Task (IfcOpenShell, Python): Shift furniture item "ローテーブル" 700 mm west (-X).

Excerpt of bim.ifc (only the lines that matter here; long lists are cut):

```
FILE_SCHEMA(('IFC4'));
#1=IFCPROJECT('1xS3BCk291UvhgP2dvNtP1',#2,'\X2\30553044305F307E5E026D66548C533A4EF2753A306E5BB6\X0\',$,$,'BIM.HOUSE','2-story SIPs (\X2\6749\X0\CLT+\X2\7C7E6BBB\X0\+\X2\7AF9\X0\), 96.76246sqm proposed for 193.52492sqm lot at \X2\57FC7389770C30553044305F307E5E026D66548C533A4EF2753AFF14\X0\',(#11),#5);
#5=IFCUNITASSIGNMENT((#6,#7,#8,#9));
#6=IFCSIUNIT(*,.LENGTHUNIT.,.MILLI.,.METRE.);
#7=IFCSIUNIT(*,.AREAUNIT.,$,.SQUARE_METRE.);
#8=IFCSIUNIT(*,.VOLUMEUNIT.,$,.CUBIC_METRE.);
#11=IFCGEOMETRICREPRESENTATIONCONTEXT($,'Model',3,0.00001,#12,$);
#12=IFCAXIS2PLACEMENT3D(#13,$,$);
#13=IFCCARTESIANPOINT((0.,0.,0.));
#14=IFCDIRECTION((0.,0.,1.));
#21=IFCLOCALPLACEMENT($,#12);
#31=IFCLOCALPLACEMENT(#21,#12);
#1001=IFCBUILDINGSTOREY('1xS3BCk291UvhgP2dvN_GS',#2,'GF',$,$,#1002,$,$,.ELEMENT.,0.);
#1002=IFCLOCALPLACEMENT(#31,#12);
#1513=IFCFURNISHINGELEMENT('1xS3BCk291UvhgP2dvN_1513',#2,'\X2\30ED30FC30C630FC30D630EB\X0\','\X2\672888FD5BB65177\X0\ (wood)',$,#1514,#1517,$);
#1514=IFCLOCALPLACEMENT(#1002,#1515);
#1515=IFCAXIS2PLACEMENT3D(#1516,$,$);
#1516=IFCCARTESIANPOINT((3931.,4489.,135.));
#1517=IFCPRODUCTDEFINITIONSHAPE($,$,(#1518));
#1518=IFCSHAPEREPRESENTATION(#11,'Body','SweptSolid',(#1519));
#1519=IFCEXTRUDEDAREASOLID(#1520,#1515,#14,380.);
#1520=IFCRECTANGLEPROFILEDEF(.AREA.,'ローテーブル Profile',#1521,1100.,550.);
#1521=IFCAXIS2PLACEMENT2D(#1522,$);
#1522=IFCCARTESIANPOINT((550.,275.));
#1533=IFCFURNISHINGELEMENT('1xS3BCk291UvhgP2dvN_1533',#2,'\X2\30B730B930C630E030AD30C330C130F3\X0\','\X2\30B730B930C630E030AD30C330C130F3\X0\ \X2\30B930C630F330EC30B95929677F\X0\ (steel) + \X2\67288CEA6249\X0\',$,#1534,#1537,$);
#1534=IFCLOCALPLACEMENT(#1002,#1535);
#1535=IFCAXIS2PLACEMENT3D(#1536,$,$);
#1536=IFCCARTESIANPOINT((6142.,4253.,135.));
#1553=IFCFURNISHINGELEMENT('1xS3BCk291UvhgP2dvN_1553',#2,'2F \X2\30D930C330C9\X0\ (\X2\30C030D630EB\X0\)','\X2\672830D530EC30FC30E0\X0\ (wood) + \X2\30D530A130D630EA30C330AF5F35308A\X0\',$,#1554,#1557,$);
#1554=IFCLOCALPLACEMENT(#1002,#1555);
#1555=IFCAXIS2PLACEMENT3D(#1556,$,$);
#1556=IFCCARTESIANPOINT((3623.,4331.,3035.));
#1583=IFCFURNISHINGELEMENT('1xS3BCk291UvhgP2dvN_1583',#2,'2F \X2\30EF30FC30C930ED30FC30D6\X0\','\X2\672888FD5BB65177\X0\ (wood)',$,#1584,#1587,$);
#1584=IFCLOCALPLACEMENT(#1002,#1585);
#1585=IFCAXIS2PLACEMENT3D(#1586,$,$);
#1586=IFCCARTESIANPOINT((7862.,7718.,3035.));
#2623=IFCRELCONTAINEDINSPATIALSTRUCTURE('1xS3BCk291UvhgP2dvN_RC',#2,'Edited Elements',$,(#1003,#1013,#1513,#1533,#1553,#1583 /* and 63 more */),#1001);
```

```python
import ifcopenshell
import ifcopenshell.api.geometry
import ifcopenshell.util.placement

model = ifcopenshell.open("bim.ifc")

item = model.by_id(1513)
matrix = ifcopenshell.util.placement.get_local_placement(item.ObjectPlacement)
matrix[0, 3] -= 700.0
ifcopenshell.api.geometry.edit_object_placement(model, product=item, matrix=matrix, is_si=False)

print(ifcopenshell.util.placement.get_local_placement(item.ObjectPlacement).round(3) + 0.0)

model.write("bim_rev.ifc")
```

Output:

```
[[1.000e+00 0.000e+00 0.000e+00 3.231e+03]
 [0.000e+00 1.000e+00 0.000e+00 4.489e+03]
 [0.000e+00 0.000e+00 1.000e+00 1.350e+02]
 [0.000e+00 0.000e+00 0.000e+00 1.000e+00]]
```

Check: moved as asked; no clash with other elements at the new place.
